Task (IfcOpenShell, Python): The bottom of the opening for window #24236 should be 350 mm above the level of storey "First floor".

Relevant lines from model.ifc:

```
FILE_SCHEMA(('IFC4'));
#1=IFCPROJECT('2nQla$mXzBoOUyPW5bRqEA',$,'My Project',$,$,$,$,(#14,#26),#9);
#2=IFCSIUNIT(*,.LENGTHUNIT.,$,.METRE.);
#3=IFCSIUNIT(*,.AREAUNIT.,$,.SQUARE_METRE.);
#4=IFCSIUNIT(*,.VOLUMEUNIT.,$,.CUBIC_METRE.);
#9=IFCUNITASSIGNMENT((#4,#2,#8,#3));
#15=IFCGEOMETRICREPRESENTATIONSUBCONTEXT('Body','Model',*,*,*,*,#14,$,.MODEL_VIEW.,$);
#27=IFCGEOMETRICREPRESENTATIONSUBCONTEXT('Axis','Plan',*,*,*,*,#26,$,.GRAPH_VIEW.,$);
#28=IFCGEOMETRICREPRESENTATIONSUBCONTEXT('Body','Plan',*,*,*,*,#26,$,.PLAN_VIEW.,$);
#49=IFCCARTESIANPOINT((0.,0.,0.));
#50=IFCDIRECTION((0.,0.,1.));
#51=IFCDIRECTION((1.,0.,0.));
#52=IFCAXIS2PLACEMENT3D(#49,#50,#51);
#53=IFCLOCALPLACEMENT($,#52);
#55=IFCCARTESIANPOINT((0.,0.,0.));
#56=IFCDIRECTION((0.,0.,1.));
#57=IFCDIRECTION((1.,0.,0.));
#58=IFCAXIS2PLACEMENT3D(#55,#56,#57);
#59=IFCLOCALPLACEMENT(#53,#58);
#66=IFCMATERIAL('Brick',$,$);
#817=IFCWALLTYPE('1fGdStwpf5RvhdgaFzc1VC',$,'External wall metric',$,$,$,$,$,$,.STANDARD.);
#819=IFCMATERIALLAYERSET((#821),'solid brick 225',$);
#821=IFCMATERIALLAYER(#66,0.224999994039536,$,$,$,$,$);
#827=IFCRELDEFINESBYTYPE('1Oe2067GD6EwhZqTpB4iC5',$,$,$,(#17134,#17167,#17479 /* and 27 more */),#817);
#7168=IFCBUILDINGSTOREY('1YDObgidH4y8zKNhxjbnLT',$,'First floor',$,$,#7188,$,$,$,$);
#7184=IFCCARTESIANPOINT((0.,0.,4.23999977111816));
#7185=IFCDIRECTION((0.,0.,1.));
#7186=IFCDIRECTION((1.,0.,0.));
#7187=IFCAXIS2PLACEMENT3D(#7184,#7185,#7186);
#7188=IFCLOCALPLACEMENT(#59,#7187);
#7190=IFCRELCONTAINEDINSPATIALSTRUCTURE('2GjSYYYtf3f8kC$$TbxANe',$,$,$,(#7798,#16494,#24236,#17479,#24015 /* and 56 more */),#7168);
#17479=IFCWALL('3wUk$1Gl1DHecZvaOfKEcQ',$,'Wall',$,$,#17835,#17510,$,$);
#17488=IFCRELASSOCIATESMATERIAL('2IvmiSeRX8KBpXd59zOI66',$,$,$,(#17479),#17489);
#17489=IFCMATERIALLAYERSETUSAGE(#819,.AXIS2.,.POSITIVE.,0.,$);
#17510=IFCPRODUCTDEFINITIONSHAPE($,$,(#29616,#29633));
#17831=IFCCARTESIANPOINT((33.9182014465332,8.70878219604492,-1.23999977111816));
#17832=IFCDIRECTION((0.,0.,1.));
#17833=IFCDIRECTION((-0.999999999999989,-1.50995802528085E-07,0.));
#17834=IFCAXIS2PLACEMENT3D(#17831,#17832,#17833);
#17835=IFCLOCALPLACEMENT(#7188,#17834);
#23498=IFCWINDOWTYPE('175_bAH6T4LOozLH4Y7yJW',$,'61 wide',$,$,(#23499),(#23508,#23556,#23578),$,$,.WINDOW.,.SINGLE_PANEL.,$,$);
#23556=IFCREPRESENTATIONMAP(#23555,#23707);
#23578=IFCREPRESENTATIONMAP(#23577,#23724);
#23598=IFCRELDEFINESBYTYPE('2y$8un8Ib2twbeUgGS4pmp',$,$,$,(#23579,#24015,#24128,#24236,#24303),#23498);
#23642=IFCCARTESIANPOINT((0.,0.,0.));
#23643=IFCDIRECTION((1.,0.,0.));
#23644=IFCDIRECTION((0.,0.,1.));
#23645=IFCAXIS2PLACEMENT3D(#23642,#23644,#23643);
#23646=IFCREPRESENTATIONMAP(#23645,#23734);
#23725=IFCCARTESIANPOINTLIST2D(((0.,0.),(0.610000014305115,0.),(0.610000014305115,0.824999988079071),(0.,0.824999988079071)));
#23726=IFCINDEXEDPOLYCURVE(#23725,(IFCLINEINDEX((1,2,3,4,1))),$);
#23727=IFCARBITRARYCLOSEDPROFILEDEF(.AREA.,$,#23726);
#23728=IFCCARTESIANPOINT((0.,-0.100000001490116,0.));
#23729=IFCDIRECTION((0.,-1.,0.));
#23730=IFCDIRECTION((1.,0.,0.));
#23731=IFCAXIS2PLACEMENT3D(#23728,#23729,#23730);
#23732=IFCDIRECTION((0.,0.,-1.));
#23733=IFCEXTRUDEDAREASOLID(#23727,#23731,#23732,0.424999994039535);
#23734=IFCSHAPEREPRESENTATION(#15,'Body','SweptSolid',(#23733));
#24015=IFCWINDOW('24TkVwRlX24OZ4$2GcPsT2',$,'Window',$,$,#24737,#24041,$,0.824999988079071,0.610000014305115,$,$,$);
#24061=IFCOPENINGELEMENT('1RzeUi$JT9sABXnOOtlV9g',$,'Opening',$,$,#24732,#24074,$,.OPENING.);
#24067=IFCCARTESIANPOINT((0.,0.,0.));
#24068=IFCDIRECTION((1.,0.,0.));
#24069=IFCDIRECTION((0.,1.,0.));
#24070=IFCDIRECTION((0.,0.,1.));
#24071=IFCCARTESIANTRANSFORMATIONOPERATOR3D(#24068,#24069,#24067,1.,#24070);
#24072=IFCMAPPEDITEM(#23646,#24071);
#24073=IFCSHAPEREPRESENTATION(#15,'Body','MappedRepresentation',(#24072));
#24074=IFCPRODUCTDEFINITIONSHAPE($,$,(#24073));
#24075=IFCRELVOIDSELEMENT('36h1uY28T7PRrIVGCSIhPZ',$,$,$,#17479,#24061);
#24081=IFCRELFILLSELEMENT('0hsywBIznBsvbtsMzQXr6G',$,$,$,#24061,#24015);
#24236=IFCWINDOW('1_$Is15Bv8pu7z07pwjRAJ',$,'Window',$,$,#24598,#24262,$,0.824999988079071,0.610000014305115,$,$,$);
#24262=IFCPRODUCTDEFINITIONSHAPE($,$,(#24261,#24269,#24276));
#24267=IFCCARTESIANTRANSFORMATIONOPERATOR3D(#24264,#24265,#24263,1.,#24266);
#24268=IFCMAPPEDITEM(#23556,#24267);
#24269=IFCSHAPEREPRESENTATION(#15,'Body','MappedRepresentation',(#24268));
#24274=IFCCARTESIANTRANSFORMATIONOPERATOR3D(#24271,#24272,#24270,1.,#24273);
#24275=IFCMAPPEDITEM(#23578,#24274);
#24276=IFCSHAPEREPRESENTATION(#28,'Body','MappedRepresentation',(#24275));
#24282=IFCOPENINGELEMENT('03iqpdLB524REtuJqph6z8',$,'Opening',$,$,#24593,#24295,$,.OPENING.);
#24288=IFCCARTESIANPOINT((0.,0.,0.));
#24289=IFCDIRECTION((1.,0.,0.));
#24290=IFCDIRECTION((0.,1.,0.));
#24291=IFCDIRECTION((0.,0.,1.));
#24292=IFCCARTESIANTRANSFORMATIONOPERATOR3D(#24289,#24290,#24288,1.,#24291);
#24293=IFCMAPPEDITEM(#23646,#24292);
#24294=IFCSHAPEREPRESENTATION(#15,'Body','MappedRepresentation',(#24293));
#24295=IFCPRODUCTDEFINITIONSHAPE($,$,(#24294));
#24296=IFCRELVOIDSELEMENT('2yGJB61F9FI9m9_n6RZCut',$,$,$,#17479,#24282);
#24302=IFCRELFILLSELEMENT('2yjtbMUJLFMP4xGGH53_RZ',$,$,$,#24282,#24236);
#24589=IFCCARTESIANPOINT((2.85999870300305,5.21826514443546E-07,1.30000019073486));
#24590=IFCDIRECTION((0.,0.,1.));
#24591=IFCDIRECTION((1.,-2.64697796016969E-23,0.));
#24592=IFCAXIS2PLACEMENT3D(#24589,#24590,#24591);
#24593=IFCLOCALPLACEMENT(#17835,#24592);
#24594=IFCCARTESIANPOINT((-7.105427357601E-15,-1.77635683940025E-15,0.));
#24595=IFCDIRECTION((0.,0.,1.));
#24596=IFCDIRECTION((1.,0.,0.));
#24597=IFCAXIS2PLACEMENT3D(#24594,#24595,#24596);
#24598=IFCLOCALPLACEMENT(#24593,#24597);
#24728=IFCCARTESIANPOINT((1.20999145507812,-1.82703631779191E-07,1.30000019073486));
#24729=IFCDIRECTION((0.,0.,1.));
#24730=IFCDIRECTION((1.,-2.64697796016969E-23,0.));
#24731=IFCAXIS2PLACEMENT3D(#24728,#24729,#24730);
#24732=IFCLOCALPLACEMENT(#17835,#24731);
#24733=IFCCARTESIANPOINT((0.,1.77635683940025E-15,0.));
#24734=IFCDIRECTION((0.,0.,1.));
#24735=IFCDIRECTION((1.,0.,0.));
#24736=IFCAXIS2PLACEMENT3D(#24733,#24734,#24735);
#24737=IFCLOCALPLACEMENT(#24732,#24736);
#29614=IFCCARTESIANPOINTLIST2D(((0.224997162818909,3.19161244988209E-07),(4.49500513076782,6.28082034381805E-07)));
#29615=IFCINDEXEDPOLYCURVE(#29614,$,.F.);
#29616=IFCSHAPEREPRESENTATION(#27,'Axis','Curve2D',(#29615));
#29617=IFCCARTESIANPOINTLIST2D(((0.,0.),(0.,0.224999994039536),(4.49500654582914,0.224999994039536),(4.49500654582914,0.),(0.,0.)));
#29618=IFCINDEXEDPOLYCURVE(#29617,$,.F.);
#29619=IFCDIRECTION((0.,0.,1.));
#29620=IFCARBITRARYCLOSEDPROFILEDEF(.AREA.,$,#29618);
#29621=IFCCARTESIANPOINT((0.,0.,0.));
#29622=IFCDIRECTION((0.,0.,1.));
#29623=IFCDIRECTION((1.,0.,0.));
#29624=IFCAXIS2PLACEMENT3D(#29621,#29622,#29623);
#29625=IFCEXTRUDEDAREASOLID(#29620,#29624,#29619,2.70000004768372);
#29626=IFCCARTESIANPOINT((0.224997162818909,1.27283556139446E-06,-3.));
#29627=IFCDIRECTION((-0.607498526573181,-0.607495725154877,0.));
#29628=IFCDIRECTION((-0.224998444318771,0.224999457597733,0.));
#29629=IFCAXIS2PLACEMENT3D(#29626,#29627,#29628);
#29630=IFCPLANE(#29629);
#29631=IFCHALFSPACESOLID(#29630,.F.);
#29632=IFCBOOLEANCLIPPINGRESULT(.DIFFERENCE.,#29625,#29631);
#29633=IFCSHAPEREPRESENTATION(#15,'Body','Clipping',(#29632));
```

```python
import numpy as np
import ifcopenshell
import ifcopenshell.api.geometry
import ifcopenshell.geom
import ifcopenshell.util.element
import ifcopenshell.util.placement
import ifcopenshell.util.shape
import ifcopenshell.util.unit

model = ifcopenshell.open("model.ifc")
unit_scale = ifcopenshell.util.unit.calculate_unit_scale(model)

window = model.by_id(24236)
opening = window.FillsVoids[0].RelatingOpeningElement
storey = ifcopenshell.util.element.get_container(window, ifc_class="IfcBuildingStorey")
level = ifcopenshell.util.placement.get_local_placement(storey.ObjectPlacement)[2, 3]

# The opening's origin need not be at the sill, so measure its lowest point.
shape = ifcopenshell.geom.create_shape(ifcopenshell.geom.settings(), opening)
bottom = ifcopenshell.util.shape.get_shape_bottom_elevation(shape, shape.geometry) / unit_scale
dz = level + 0.35 / unit_scale - bottom

shift = np.array([0.0, 0.0, dz])
# The window is placed relative to its opening, so it follows when the opening moves.
matrix = ifcopenshell.util.placement.get_local_placement(opening.ObjectPlacement)
matrix[:3, 3] += shift
ifcopenshell.api.geometry.edit_object_placement(
    model, product=opening, matrix=matrix, is_si=False, should_transform_children=True
)

print(f"moved by {dz * unit_scale:+.3f} m")

model.write("model_edited.ifc")
```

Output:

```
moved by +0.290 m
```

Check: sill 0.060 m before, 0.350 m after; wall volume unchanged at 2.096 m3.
